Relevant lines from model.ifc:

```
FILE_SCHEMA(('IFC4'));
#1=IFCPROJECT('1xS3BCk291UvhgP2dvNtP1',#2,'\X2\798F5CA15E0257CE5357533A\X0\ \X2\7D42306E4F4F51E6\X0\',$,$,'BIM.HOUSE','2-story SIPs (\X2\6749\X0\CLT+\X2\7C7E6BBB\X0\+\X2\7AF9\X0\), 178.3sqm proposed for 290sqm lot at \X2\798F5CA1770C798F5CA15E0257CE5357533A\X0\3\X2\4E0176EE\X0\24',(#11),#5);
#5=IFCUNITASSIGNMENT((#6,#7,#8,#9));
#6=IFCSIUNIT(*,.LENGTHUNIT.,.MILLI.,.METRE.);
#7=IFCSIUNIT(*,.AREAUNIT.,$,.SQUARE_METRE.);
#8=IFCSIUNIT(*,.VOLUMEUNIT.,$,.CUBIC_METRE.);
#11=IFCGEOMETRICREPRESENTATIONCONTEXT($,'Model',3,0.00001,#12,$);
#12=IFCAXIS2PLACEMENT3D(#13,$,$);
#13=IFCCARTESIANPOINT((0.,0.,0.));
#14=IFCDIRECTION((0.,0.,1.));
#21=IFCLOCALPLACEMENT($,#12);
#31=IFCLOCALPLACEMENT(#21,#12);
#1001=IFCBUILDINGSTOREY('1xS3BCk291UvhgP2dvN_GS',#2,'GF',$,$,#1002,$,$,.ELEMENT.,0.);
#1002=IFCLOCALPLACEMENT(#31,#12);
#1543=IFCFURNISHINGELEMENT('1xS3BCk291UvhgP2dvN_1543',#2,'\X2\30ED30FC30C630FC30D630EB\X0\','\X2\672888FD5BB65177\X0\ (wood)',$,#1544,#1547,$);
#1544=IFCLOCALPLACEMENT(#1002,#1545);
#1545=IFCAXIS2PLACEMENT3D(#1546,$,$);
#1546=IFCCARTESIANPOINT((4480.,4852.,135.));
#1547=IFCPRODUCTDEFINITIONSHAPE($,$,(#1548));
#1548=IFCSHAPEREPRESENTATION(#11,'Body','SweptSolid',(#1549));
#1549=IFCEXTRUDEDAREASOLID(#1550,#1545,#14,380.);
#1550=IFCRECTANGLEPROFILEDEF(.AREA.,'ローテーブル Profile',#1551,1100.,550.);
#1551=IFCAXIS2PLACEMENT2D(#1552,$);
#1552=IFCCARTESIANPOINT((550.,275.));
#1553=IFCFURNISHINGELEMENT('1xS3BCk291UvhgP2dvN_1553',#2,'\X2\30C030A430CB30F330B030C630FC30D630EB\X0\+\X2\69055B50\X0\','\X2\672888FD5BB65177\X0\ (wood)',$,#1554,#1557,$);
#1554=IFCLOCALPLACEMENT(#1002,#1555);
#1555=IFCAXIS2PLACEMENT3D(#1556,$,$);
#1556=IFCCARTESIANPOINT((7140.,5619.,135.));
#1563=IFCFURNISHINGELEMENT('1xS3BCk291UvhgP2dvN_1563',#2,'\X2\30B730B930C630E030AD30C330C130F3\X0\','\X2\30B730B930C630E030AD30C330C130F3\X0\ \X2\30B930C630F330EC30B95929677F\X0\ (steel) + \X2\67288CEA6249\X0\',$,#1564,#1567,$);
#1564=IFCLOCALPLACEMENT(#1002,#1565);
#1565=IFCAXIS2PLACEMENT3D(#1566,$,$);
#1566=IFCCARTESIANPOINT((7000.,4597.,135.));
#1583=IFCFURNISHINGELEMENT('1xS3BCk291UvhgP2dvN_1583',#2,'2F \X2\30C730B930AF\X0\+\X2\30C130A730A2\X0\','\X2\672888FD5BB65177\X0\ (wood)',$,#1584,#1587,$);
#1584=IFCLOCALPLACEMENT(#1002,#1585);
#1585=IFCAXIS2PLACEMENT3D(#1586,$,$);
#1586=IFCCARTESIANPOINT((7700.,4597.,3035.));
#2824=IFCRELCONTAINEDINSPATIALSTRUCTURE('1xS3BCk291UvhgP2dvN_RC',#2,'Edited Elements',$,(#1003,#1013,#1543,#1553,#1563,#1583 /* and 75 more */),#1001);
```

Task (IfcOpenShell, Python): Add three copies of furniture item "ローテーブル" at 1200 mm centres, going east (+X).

```python
import numpy as np
import ifcopenshell
import ifcopenshell.api.geometry
import ifcopenshell.api.root
import ifcopenshell.util.element
import ifcopenshell.util.placement

model = ifcopenshell.open("model.ifc")


def reuse_history(source, copy):
    """copy_class also copies each property set's owner history, people and application; keep the originals."""
    for rel in copy.IsDefinedBy:
        if rel.is_a("IfcRelDefinesByProperties") and (history := rel.RelatingPropertyDefinition.OwnerHistory):
            rel.RelatingPropertyDefinition.OwnerHistory = source.OwnerHistory
            ifcopenshell.util.element.remove_deep2(model, history)


source = model.by_id(1543)
base = ifcopenshell.util.placement.get_local_placement(source.ObjectPlacement)
step = np.array([1.0, 0.0, 0.0]) * 1200.0

for i in range(1, 4):
    copy = ifcopenshell.api.root.copy_class(model, product=source)
    copy.Representation = ifcopenshell.util.element.copy_deep(
        model, source.Representation, exclude=["IfcGeometricRepresentationContext", "IfcRepresentationMap"]
    )
    reuse_history(source, copy)
    matrix = base.copy()
    matrix[:3, 3] += i * step
    print("added at", matrix[:3, 3].round(3) + 0.0)
    ifcopenshell.api.geometry.edit_object_placement(model, product=copy, matrix=matrix, is_si=False)

model.write("model_edited.ifc")
```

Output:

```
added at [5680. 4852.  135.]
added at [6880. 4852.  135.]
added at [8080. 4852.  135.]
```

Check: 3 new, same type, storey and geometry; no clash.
